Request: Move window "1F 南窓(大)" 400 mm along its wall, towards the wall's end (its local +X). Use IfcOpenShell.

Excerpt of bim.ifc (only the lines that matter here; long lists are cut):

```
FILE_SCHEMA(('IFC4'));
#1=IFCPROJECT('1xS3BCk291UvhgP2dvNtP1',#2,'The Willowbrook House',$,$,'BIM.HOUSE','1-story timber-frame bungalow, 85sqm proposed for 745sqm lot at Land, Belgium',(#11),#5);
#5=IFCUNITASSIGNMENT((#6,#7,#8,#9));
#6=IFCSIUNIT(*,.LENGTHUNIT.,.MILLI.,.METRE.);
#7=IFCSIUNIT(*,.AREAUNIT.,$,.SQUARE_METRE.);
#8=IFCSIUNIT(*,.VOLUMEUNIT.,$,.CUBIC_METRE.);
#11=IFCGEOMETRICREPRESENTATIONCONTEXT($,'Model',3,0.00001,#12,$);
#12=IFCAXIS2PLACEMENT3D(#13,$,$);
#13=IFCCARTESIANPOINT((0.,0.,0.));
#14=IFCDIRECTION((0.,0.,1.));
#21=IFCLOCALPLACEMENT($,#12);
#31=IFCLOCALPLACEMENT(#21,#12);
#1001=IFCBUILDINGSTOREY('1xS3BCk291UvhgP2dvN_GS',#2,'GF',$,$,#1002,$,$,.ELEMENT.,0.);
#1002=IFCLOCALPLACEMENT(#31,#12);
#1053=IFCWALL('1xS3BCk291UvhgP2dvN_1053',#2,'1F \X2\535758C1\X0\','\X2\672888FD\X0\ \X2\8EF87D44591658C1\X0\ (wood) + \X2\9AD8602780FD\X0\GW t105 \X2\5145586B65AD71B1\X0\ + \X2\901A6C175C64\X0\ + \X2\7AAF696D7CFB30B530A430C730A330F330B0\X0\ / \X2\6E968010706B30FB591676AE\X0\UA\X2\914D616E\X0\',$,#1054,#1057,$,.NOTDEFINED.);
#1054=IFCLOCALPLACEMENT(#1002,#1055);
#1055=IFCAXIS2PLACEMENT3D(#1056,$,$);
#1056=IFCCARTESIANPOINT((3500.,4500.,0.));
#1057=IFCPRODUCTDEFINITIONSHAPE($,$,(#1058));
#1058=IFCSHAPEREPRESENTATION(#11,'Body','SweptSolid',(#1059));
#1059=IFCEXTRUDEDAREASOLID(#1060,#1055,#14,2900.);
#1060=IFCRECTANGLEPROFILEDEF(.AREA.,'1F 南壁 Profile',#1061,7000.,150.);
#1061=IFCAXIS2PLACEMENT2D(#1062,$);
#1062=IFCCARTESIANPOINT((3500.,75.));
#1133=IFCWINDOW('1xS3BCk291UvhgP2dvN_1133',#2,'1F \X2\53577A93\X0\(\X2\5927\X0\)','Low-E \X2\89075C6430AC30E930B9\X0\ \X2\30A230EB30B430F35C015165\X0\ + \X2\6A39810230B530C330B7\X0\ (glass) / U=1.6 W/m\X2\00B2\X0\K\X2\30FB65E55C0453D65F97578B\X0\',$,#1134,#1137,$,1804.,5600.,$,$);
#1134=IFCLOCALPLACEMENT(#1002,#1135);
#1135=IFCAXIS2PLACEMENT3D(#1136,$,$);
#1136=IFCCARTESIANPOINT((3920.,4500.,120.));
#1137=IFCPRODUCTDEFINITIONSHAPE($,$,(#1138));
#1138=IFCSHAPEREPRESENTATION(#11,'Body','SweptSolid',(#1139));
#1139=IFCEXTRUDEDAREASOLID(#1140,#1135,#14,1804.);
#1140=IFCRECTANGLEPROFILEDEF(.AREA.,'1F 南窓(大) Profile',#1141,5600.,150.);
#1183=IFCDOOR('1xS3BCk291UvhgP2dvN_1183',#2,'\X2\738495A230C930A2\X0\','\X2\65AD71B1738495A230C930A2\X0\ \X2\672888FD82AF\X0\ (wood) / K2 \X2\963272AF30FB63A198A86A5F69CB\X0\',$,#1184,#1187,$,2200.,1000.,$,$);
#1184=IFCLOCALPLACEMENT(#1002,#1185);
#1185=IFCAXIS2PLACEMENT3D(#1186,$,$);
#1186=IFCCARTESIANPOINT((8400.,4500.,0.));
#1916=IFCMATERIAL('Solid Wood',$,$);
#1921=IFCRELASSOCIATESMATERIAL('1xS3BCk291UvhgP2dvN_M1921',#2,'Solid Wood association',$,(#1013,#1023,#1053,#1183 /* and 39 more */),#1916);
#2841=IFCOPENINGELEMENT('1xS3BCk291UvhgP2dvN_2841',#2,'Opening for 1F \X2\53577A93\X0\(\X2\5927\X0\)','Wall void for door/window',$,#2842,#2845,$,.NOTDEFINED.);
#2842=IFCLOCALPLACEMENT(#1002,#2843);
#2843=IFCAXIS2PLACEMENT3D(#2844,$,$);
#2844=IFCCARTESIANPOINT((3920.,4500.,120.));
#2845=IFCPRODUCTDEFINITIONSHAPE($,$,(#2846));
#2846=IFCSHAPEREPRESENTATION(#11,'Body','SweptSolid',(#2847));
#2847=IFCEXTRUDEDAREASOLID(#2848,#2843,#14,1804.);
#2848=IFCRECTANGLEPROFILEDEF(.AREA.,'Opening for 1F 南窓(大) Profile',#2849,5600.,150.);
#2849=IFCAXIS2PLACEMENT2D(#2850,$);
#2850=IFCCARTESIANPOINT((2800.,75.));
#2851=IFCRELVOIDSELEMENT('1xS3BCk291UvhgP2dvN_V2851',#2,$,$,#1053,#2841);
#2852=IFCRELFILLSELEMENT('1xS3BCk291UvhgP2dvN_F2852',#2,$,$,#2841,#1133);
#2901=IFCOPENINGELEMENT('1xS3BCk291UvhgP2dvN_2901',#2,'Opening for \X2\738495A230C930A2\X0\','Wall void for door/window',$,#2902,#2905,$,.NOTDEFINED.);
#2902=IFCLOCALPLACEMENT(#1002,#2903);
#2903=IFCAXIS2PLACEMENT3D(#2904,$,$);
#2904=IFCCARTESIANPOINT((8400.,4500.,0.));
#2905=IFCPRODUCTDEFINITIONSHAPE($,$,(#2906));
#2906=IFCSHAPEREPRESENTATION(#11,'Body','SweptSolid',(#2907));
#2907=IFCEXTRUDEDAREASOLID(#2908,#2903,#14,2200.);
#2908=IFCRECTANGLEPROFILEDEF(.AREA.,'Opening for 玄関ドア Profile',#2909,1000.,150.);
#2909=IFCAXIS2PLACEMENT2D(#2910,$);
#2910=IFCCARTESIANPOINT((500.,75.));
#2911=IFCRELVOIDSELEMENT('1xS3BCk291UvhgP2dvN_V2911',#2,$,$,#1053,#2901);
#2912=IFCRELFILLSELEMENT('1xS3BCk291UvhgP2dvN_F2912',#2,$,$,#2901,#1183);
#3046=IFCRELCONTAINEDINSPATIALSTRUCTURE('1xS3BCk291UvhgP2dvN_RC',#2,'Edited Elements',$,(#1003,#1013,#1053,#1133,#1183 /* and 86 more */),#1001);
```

```python
import ifcopenshell
import ifcopenshell.api.geometry
import ifcopenshell.util.placement

model = ifcopenshell.open("bim.ifc")

window = model.by_id(1133)
opening = window.FillsVoids[0].RelatingOpeningElement
wall = opening.VoidsElements[0].RelatingBuildingElement

wall_matrix = ifcopenshell.util.placement.get_local_placement(wall.ObjectPlacement)
shift = wall_matrix[:3, 0] * 400.0
before = ifcopenshell.util.placement.get_local_placement(window.ObjectPlacement)[:3, 3].copy()

# The window is not placed relative to its opening, so move both.
for product in (opening, window):
    matrix = ifcopenshell.util.placement.get_local_placement(product.ObjectPlacement)
    matrix[:3, 3] += shift
    ifcopenshell.api.geometry.edit_object_placement(model, product=product, matrix=matrix, is_si=False)

after = ifcopenshell.util.placement.get_local_placement(window.ObjectPlacement)[:3, 3]
print("window moved by", (after - before).round(3) + 0.0)

model.write("bim_rev.ifc")
```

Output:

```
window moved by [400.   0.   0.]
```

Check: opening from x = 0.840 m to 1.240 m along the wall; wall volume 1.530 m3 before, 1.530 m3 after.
